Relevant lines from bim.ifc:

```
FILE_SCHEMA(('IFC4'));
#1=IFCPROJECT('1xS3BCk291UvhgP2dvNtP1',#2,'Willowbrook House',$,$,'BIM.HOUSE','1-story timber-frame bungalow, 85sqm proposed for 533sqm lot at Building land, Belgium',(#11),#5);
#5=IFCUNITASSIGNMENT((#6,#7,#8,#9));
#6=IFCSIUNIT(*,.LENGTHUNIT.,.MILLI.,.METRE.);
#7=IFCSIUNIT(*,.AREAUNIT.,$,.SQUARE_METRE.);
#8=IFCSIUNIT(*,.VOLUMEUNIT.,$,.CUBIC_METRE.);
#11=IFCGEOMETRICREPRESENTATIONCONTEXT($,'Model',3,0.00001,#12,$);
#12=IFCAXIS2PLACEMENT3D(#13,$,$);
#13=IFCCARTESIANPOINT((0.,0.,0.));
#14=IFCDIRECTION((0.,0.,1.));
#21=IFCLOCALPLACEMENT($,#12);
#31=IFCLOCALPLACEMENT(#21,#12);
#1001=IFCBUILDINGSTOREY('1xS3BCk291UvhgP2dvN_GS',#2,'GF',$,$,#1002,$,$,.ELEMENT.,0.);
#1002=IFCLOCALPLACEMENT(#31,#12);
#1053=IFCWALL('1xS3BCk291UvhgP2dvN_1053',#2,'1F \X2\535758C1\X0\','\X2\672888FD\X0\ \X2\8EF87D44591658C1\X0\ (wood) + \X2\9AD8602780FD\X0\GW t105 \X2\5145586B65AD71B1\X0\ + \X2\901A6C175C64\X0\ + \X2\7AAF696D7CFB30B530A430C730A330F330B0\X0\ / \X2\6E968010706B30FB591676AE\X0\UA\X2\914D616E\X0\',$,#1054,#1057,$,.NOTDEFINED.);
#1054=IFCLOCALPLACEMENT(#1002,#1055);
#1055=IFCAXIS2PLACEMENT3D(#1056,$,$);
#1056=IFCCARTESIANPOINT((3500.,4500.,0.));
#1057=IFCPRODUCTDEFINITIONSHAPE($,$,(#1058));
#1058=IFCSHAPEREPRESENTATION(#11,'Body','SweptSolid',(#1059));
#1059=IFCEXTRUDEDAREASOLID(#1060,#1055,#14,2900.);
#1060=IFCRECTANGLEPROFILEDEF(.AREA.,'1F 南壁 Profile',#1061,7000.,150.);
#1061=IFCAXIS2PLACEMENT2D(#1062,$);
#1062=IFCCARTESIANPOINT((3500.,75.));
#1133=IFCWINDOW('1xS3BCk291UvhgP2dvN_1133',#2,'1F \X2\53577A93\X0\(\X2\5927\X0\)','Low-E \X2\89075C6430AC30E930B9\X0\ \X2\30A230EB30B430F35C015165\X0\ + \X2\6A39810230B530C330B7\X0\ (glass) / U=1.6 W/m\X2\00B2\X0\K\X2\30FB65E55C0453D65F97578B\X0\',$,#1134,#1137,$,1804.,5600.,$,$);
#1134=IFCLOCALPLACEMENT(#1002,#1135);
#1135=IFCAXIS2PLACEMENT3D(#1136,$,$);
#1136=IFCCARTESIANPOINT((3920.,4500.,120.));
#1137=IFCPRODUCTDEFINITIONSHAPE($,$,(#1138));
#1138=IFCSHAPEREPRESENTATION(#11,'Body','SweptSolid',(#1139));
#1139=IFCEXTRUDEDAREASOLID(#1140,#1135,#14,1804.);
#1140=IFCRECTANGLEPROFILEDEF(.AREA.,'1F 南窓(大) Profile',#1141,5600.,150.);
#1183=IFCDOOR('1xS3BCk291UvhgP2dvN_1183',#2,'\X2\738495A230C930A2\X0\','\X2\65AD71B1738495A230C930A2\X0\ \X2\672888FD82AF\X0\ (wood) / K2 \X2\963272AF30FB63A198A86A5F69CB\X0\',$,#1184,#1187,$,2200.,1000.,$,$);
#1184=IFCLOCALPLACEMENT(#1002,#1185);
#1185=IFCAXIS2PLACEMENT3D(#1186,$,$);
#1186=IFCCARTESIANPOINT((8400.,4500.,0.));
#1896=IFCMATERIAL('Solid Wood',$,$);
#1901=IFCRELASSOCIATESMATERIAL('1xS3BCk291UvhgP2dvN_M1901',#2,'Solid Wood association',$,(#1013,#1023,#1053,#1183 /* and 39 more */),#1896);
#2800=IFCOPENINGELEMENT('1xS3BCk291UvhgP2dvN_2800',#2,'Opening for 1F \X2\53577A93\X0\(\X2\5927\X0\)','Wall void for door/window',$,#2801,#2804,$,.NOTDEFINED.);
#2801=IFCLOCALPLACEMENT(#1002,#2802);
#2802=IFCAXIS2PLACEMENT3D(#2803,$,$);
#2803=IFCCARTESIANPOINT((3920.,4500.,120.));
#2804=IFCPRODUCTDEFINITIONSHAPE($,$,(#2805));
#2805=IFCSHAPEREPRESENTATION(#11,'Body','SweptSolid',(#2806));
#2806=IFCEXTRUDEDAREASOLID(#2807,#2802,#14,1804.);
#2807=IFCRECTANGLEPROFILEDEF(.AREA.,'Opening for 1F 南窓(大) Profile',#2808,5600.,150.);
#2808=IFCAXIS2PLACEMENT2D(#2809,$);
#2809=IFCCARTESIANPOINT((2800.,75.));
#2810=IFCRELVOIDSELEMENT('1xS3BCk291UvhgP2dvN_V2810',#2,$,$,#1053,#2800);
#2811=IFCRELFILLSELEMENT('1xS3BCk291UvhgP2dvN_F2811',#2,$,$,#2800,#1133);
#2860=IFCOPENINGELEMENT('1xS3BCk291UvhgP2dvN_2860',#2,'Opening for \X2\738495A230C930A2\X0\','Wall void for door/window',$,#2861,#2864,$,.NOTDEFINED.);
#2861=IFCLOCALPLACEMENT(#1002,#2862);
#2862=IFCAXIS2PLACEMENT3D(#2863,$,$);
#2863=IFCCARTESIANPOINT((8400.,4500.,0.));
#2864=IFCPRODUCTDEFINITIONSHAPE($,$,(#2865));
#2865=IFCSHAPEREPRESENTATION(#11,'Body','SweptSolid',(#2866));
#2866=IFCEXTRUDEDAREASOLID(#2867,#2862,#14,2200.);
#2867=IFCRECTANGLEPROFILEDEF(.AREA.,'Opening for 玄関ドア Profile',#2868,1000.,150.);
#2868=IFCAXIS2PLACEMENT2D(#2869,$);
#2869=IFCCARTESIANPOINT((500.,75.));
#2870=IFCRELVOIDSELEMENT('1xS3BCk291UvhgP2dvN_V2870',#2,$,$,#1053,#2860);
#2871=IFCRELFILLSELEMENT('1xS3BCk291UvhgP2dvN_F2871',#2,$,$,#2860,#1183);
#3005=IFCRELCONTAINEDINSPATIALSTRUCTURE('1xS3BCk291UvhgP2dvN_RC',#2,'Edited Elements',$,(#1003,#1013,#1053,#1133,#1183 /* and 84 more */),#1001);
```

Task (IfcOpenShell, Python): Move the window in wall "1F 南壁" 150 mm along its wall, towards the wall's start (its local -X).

```python
import ifcopenshell
import ifcopenshell.api.geometry
import ifcopenshell.util.placement

model = ifcopenshell.open("bim.ifc")

window = model.by_guid("1xS3BCk291UvhgP2dvN_1133")
opening = window.FillsVoids[0].RelatingOpeningElement
wall = opening.VoidsElements[0].RelatingBuildingElement

wall_matrix = ifcopenshell.util.placement.get_local_placement(wall.ObjectPlacement)
shift = wall_matrix[:3, 0] * -150.0
before = ifcopenshell.util.placement.get_local_placement(window.ObjectPlacement)[:3, 3].copy()

# The window is not placed relative to its opening, so move both.
for product in (opening, window):
    matrix = ifcopenshell.util.placement.get_local_placement(product.ObjectPlacement)
    matrix[:3, 3] += shift
    ifcopenshell.api.geometry.edit_object_placement(model, product=product, matrix=matrix, is_si=False)

after = ifcopenshell.util.placement.get_local_placement(window.ObjectPlacement)[:3, 3]
print("window moved by", (after - before).round(3) + 0.0)

model.write("bim_v2.ifc")
```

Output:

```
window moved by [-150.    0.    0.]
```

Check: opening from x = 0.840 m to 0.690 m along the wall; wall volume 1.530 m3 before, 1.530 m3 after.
